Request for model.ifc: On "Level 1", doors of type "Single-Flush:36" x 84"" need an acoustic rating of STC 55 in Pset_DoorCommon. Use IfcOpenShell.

First a look at what the model holds.

```python
import ifcopenshell
import ifcopenshell.util.element

model = ifcopenshell.open("model.ifc")
print(model.schema)
storey = next(s for s in model.by_type("IfcBuildingStorey") if s.Name == "Level 1")
doors = [e for e in ifcopenshell.util.element.get_decomposition(storey) if e.is_a("IfcDoor")]
seen = {}
for e in doors:
    element_type = ifcopenshell.util.element.get_type(e)
    key = (element_type.Name if element_type != e and element_type else None, ifcopenshell.util.element.get_pset(e, "Pset_DoorCommon", "AcousticRating"))
    seen[key] = seen.get(key, 0) + 1
for (name, value), count in sorted(seen.items(), key=str):
    print(count, "x", name, "|", value)
```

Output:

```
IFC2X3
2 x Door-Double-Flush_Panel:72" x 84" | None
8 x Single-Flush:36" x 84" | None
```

```python
import ifcopenshell
import ifcopenshell.api.pset
import ifcopenshell.util.element

model = ifcopenshell.open("model.ifc")

storey = next(s for s in model.by_type("IfcBuildingStorey") if s.Name == "Level 1")
doors = [e for e in ifcopenshell.util.element.get_decomposition(storey) if e.is_a("IfcDoor")]

count = 0
for e in doors:
    element_type = ifcopenshell.util.element.get_type(e)
    if element_type in (None, e) or element_type.Name != 'Single-Flush:36" x 84"':
        continue
    # add_pset returns the element's existing set when there is one.
    pset = ifcopenshell.api.pset.add_pset(model, product=e, name="Pset_DoorCommon")
    ifcopenshell.api.pset.edit_pset(model, pset=pset, properties={"AcousticRating": "STC 55"})
    count += 1

print(count, "doors updated")

model.write("model_edited.ifc")
```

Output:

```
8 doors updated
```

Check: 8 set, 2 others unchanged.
